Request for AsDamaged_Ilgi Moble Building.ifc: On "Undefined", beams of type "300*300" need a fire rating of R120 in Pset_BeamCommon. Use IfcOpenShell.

First a look at what the model holds.

```python
import ifcopenshell
import ifcopenshell.util.element

model = ifcopenshell.open("AsDamaged_Ilgi Moble Building.ifc")
print(model.schema)
storey = next(s for s in model.by_type("IfcBuildingStorey") if s.Name == "Undefined")
beams = [e for e in ifcopenshell.util.element.get_decomposition(storey) if e.is_a("IfcBeam")]
seen = {}
for e in beams:
    element_type = ifcopenshell.util.element.get_type(e)
    key = (element_type.Name if element_type != e and element_type else None, ifcopenshell.util.element.get_pset(e, "Pset_BeamCommon", "FireRating"))
    seen[key] = seen.get(key, 0) + 1
for (name, value), count in sorted(seen.items(), key=str):
    print(count, "x", name, "|", value)
```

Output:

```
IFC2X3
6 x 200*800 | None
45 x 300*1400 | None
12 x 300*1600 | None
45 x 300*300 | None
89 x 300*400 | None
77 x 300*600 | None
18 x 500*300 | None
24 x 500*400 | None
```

```python
import ifcopenshell
import ifcopenshell.api.pset
import ifcopenshell.util.element

model = ifcopenshell.open("AsDamaged_Ilgi Moble Building.ifc")

storey = next(s for s in model.by_type("IfcBuildingStorey") if s.Name == "Undefined")
beams = [e for e in ifcopenshell.util.element.get_decomposition(storey) if e.is_a("IfcBeam")]

count = 0
for e in beams:
    element_type = ifcopenshell.util.element.get_type(e)
    if element_type in (None, e) or element_type.Name != "300*300":
        continue
    # add_pset returns the element's existing set when there is one.
    pset = ifcopenshell.api.pset.add_pset(model, product=e, name="Pset_BeamCommon")
    ifcopenshell.api.pset.edit_pset(model, pset=pset, properties={"FireRating": "R120"})
    count += 1

print(count, "beams updated")

model.write("AsDamaged_Ilgi Moble Building_updated.ifc")
```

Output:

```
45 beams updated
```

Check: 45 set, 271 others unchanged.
